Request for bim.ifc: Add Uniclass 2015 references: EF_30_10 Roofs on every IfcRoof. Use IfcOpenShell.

First a look at what the model holds.

```python
import ifcopenshell

model = ifcopenshell.open("bim.ifc")
print(model.schema)
print("classifications:", [c.Name for c in model.by_type("IfcClassification")])
for ifc_class in ("IfcDoor", "IfcRoof", "IfcStair", "IfcWall", "IfcWindow"):
    print(ifc_class, len(model.by_type(ifc_class)))
```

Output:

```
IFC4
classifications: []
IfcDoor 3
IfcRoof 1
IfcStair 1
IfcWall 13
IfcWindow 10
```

```python
import ifcopenshell
import ifcopenshell.api.classification

model = ifcopenshell.open("bim.ifc")

system = ifcopenshell.api.classification.add_classification(model, classification="Uniclass 2015")

codes = {
    "IfcRoof": ("EF_30_10", "Roofs"),
}
for ifc_class, (code, name) in codes.items():
    products = model.by_type(ifc_class)
    ifcopenshell.api.classification.add_reference(
        model, products=products, classification=system, identification=code, name=name
    )
    print(code, len(products))

model.write("bim_updated.ifc")
```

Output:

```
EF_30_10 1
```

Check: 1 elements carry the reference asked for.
